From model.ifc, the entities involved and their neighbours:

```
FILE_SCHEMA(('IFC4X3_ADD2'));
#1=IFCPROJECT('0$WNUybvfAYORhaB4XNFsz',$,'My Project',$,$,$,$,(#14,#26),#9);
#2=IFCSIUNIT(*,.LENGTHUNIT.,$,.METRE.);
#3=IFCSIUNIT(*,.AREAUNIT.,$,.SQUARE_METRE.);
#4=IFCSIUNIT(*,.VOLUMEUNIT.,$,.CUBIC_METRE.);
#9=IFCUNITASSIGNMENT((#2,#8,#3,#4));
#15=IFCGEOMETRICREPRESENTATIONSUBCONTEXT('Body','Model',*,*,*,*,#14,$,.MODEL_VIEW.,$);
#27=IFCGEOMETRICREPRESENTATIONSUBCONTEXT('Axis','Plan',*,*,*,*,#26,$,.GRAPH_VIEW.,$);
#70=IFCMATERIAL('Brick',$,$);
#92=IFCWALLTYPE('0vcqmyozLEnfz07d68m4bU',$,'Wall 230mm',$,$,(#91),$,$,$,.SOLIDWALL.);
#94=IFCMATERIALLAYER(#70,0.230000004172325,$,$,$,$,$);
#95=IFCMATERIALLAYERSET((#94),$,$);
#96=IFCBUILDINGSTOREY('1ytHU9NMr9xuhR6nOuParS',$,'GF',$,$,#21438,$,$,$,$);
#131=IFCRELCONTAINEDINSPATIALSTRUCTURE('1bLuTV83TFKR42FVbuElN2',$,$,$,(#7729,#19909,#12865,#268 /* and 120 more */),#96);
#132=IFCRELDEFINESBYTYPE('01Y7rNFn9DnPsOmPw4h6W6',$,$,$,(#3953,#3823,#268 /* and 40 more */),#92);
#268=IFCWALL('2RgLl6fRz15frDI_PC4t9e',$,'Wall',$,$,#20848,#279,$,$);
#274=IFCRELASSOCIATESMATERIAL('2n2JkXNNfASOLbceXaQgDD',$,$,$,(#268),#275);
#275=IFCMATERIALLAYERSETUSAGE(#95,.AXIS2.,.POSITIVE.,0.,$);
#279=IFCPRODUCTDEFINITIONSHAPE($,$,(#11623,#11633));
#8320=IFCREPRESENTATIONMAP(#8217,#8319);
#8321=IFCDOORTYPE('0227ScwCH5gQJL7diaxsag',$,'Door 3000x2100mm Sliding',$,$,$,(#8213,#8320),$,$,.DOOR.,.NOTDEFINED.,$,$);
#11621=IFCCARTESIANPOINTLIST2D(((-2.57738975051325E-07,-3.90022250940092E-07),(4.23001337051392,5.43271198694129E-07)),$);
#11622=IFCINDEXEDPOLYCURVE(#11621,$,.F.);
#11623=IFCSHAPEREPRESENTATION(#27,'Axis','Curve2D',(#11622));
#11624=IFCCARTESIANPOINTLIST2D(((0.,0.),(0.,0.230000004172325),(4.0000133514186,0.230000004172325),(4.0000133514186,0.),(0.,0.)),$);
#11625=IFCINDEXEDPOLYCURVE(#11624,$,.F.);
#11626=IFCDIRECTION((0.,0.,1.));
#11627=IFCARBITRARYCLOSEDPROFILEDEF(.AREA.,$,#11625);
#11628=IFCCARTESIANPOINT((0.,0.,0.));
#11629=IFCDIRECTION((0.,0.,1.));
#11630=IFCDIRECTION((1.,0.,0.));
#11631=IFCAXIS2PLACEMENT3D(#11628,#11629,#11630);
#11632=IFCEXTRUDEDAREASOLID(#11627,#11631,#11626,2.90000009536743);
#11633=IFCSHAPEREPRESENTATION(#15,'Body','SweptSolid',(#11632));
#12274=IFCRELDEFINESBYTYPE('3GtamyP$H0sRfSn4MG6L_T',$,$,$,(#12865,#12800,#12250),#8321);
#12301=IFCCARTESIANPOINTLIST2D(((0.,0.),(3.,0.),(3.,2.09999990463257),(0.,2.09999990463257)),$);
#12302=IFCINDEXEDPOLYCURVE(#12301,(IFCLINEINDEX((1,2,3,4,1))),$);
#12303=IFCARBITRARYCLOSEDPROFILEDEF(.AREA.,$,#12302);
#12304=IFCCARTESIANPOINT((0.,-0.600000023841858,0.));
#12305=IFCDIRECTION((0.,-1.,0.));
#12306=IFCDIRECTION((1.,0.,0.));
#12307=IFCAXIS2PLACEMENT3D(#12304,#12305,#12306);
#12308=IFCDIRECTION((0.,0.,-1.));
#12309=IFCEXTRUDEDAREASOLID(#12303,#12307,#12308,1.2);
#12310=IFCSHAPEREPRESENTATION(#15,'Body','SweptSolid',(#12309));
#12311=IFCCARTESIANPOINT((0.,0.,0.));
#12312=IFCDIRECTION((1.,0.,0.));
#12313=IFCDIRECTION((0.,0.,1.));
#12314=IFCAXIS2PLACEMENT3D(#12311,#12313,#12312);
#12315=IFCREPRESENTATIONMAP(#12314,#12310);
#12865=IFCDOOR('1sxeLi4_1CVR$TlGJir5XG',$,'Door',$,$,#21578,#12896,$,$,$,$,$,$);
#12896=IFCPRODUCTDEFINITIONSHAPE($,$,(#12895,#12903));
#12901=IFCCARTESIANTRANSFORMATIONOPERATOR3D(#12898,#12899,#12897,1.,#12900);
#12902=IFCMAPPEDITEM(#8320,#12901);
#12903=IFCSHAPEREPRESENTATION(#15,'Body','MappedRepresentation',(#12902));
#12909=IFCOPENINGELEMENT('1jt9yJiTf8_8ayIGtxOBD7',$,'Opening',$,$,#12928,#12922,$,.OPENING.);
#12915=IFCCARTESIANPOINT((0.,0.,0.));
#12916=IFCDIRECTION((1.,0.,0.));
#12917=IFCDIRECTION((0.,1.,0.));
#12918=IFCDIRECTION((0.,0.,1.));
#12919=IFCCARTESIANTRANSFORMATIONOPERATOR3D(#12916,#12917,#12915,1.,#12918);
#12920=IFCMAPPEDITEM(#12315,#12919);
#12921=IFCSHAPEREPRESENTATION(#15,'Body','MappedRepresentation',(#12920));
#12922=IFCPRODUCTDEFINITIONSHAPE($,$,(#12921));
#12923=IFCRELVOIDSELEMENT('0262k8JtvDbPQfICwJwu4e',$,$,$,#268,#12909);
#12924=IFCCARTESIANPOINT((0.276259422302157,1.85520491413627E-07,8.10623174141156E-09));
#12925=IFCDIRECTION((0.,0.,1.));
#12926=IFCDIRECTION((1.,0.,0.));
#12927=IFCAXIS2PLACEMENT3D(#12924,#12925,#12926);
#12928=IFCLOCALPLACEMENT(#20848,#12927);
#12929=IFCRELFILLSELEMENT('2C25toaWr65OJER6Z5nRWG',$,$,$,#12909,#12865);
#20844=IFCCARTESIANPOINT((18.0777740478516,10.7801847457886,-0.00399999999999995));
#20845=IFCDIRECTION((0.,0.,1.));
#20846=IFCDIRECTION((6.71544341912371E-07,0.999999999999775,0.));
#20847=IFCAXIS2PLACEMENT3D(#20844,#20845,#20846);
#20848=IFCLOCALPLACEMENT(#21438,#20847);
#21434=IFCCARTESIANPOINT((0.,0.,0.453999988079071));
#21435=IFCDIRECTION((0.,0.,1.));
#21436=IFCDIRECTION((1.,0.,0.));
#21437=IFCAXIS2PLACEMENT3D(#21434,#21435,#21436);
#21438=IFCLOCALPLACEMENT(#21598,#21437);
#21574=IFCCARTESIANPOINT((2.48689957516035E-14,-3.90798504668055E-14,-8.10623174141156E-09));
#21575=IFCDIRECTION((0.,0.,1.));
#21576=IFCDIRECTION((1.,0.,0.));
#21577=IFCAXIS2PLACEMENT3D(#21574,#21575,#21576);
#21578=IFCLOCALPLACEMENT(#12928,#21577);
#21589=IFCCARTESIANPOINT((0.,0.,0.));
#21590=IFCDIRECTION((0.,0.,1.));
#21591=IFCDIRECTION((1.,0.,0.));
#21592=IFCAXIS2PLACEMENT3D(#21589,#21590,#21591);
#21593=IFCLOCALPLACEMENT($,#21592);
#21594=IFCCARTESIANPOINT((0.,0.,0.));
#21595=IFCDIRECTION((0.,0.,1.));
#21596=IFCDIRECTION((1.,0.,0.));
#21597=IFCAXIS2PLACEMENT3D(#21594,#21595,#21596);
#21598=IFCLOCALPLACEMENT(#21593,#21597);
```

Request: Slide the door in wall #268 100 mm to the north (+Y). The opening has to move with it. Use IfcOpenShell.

```python
import ifcopenshell
import ifcopenshell.api.geometry
import ifcopenshell.util.placement
import ifcopenshell.util.unit

model = ifcopenshell.open("model.ifc")
unit_scale = ifcopenshell.util.unit.calculate_unit_scale(model)

door = model.by_guid("1sxeLi4_1CVR$TlGJir5XG")
opening = door.FillsVoids[0].RelatingOpeningElement
wall = opening.VoidsElements[0].RelatingBuildingElement

wall_matrix = ifcopenshell.util.placement.get_local_placement(wall.ObjectPlacement)
shift = wall_matrix[:3, 0] * 0.1 / unit_scale
before = ifcopenshell.util.placement.get_local_placement(door.ObjectPlacement)[:3, 3].copy()

# The door is placed relative to its opening, so it follows when the opening moves.
matrix = ifcopenshell.util.placement.get_local_placement(opening.ObjectPlacement)
matrix[:3, 3] += shift
ifcopenshell.api.geometry.edit_object_placement(
    model, product=opening, matrix=matrix, is_si=False, should_transform_children=True
)

after = ifcopenshell.util.placement.get_local_placement(door.ObjectPlacement)[:3, 3]
print("door moved by", (after - before).round(3) + 0.0)

model.write("model_v2.ifc")
```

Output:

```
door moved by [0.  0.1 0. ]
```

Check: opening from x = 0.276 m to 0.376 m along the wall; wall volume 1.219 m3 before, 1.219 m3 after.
